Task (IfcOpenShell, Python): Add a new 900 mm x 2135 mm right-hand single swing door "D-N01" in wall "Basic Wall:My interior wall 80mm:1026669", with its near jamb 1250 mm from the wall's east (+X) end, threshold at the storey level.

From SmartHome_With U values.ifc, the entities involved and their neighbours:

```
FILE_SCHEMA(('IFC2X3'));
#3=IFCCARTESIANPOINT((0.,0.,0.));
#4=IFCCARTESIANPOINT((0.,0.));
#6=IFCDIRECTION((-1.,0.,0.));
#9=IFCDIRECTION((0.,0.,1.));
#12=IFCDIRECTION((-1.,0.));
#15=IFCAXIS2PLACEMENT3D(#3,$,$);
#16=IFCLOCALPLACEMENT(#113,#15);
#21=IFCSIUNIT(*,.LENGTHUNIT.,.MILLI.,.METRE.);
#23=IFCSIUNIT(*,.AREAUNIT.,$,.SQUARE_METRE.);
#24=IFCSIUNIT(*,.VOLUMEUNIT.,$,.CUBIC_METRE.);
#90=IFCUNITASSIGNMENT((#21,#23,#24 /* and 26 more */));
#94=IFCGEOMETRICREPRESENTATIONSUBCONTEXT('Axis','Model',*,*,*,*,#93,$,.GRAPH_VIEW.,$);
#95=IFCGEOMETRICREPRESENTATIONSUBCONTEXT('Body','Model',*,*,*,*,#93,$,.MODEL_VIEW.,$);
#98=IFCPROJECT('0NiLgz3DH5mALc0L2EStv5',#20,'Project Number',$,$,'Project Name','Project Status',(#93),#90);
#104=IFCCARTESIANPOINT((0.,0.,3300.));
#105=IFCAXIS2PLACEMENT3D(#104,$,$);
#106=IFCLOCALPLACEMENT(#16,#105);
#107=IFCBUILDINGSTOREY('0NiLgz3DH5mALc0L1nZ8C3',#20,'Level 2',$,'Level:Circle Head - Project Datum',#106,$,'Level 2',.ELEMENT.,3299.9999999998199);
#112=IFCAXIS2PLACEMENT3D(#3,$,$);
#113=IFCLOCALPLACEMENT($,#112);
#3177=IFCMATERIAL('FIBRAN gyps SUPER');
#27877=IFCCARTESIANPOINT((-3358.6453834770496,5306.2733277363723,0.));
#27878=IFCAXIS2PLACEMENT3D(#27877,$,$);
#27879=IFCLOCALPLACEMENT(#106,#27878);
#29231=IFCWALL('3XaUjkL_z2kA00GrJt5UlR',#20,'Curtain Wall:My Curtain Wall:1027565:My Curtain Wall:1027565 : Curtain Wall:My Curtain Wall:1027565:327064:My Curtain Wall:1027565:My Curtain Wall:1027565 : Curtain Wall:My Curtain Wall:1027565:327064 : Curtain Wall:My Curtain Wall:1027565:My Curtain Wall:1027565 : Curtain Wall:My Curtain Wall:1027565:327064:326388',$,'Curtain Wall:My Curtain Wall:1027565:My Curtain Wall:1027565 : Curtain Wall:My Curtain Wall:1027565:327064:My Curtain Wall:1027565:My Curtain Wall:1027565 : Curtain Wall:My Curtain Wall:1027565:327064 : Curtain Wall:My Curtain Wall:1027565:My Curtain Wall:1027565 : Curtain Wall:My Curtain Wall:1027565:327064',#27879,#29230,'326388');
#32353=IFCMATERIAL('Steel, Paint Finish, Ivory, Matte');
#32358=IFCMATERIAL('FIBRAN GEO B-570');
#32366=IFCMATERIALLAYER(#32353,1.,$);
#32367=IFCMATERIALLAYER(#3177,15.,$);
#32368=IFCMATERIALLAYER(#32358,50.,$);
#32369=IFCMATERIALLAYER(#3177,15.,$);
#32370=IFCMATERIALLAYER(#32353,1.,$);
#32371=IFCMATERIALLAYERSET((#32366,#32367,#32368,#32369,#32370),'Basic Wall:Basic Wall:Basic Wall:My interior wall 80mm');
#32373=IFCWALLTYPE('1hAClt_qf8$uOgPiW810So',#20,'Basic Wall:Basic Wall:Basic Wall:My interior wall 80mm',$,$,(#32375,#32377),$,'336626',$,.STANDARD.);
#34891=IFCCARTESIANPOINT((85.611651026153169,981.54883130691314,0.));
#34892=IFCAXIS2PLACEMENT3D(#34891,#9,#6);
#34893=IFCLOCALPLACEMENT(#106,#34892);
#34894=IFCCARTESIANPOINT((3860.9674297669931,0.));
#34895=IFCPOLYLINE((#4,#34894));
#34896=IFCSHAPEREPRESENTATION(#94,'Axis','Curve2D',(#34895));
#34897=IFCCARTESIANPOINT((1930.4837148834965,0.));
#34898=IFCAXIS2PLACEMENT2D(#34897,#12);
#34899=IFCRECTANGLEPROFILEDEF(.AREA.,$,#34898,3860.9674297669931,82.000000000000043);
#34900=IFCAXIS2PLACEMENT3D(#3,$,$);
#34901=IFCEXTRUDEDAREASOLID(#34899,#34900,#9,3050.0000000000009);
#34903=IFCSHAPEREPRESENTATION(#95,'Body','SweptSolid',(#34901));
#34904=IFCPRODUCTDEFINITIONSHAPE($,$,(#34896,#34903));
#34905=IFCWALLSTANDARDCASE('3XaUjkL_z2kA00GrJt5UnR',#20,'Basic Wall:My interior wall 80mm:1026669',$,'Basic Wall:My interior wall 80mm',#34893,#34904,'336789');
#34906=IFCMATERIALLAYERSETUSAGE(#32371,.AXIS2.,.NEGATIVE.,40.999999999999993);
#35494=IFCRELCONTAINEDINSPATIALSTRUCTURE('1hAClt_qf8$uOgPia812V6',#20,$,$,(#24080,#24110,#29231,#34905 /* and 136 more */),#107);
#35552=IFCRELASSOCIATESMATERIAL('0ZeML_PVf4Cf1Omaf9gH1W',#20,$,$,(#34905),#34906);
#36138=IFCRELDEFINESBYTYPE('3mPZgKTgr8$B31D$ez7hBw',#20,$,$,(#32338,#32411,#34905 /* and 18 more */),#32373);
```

```python
import numpy as np
import ifcopenshell
import ifcopenshell.api.feature
import ifcopenshell.api.geometry
import ifcopenshell.api.root
import ifcopenshell.api.spatial
import ifcopenshell.api.type
import ifcopenshell.geom
import ifcopenshell.util.element
import ifcopenshell.util.placement
import ifcopenshell.util.representation
import ifcopenshell.util.shape
import ifcopenshell.util.unit

model = ifcopenshell.open("SmartHome_With U values.ifc")
unit_scale = ifcopenshell.util.unit.calculate_unit_scale(model)
settings = ifcopenshell.geom.settings()


def volume(element):
    """Net volume in cubic metres, openings subtracted."""
    shape = ifcopenshell.geom.create_shape(settings, element)
    return ifcopenshell.util.shape.get_volume(shape.geometry)


wall = model.by_guid("3XaUjkL_z2kA00GrJt5UnR")
storey = ifcopenshell.util.element.get_container(wall, ifc_class="IfcBuildingStorey")
context = ifcopenshell.util.representation.get_context(model, "Model", "Body", "MODEL_VIEW")
before = volume(wall)

width, height, from_end, sill = 0.9, 2.135, 1.25, 0.0  # metres

# The wall runs along its own X axis, and the end named is its -X end.
wall_shape = ifcopenshell.geom.create_shape(settings, wall)
x, y, z = ifcopenshell.util.shape.get_vertices(wall_shape.geometry).T
start = x.min() + from_end
face, thickness = float(y.min()), float(y.max() - y.min())
wall_matrix = ifcopenshell.util.placement.get_local_placement(wall.ObjectPlacement)
level = ifcopenshell.util.placement.get_local_placement(storey.ObjectPlacement)[2, 3]


def in_wall(x, y):
    """Placement at x, y metres in the wall's axes, at sill height."""
    matrix = wall_matrix.copy()
    matrix[:, 3] = wall_matrix @ np.array([x / unit_scale, y / unit_scale, 0.0, 1.0])
    matrix[2, 3] = level + sill / unit_scale
    return matrix


# Opening: a box that overshoots both wall faces by 50 mm.
opening = ifcopenshell.api.root.create_entity(model, ifc_class="IfcOpeningElement")
box = ifcopenshell.api.geometry.add_wall_representation(
    model, context=context, length=width, height=height, thickness=thickness + 0.1
)
ifcopenshell.api.geometry.assign_representation(model, product=opening, representation=box)
ifcopenshell.api.geometry.edit_object_placement(model, product=opening, matrix=in_wall(start, face - 0.05), is_si=False)
ifcopenshell.api.feature.add_feature(model, feature=opening, element=wall)

door = ifcopenshell.api.root.create_entity(model, ifc_class="IfcDoor", name="D-N01")
door.OverallWidth, door.OverallHeight = width / unit_scale, height / unit_scale
body = ifcopenshell.api.geometry.add_door_representation(
    model,
    context=context,
    overall_width=door.OverallWidth,
    overall_height=door.OverallHeight,
    operation_type="SINGLE_SWING_RIGHT",
    lining_properties={"LiningDepth": thickness / unit_scale, "ThresholdDepth": thickness / unit_scale},
)
ifcopenshell.api.geometry.assign_representation(model, product=door, representation=body)
ifcopenshell.api.spatial.assign_container(model, products=[door], relating_structure=storey)
fills = ifcopenshell.api.feature.add_filling(model, opening=opening, element=door)
fills.OwnerHistory = door.OwnerHistory  # required in IFC2X3

# IFC2X3 keeps the operation on the door style.
style = ifcopenshell.api.root.create_entity(model, ifc_class="IfcDoorStyle", name="D-N01")
style.OperationType, style.ConstructionType = "SINGLE_SWING_RIGHT", "NOTDEFINED"
style.ParameterTakesPrecedence = style.Sizeable = False
ifcopenshell.api.type.assign_type(model, related_objects=[door], relating_type=style)

# The lining spans the wall, so the door starts at the wall face.
ifcopenshell.api.geometry.edit_object_placement(model, product=door, matrix=in_wall(start, face), is_si=False)

after = volume(wall)

print(f"wall volume {before:.3f} -> {after:.3f} m3")

model.write("SmartHome_With U values_updated.ifc")
```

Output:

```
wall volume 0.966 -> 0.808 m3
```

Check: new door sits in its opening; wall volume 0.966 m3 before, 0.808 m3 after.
